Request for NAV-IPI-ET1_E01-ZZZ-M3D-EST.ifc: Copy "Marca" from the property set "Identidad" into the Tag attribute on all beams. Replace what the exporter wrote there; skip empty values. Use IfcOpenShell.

First a look at what the model holds.

```python
import ifcopenshell
import ifcopenshell.util.element

model = ifcopenshell.open("NAV-IPI-ET1_E01-ZZZ-M3D-EST.ifc")
print(model.schema)
beams = model.by_type("IfcBeam")
print(len(beams), "beams")
for e in beams[:8]:
    source = ifcopenshell.util.element.get_pset(e, "Identidad", "Marca")
    target = e.Tag
    print(e.id(), repr(source), repr(target), sep=" | ")
```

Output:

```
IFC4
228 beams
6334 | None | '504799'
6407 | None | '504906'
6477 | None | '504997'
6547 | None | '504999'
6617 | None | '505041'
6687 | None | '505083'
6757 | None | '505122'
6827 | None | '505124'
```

```python
import ifcopenshell
import ifcopenshell.util.element

model = ifcopenshell.open("NAV-IPI-ET1_E01-ZZZ-M3D-EST.ifc")

count = 0
for e in model.by_type("IfcBeam"):
    value = ifcopenshell.util.element.get_pset(e, "Identidad", "Marca")
    current = e.Tag
    if not value or not value.strip() or current == value:
        continue
    e.Tag = value
    count += 1

print(count, "beams updated")

model.write("NAV-IPI-ET1_E01-ZZZ-M3D-EST-out.ifc")
```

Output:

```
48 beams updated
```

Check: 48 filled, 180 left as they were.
